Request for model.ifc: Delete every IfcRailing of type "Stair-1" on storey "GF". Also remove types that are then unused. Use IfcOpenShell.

First a look at what the model holds.

```python
import ifcopenshell
import ifcopenshell.util.element

model = ifcopenshell.open("model.ifc")
print(model.schema)
storey = next(s for s in model.by_type("IfcBuildingStorey") if s.Name == "GF")
railings = [e for e in ifcopenshell.util.element.get_decomposition(storey) if e.is_a("IfcRailing")]
seen = {}
for e in railings:
    element_type = ifcopenshell.util.element.get_type(e)
    name = element_type.Name if element_type not in (None, e) else None
    seen[name] = seen.get(name, 0) + 1
for name, count in sorted(seen.items(), key=str):
    print(count, "x", name)
```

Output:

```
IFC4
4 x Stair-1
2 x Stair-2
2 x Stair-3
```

```python
import ifcopenshell
import ifcopenshell.api.root
import ifcopenshell.util.element

model = ifcopenshell.open("model.ifc")

storey = next(s for s in model.by_type("IfcBuildingStorey") if s.Name == "GF")
railings = [e for e in ifcopenshell.util.element.get_decomposition(storey) if e.is_a("IfcRailing")]
targets = [e for e in railings if (t := ifcopenshell.util.element.get_type(e)) not in (None, e) and t.Name == "Stair-1"]
types = {ifcopenshell.util.element.get_type(e) for e in targets} - {None, *targets}

for e in targets:
    ifcopenshell.api.root.remove_product(model, product=e)
print(len(targets), "removed")

unused = [t for t in types if not ifcopenshell.util.element.get_types(t)]
for t in unused:
    ifcopenshell.api.root.remove_product(model, product=t)
print(len(unused), "unused types removed")

model.write("model_v2.ifc")
```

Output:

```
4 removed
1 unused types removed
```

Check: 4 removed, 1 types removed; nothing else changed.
